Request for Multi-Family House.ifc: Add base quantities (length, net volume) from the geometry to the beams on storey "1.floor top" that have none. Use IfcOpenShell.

First a look at what the model holds.

```python
import ifcopenshell
import ifcopenshell.util.element
import ifcopenshell.util.unit

model = ifcopenshell.open("Multi-Family House.ifc")
print(model.schema)
for unit_type in ("LENGTHUNIT", "AREAUNIT", "VOLUMEUNIT"):
    print(unit_type, ifcopenshell.util.unit.calculate_unit_scale(model, unit_type))
storey = next(s for s in model.by_type("IfcBuildingStorey") if s.Name == "1.floor top")
beams = [e for e in ifcopenshell.util.element.get_decomposition(storey) if e.is_a("IfcBeam")]
for e in sorted(beams, key=lambda e: e.id()):
    print(e.id(), e.is_a(), e.Name, list(ifcopenshell.util.element.get_psets(e, qtos_only=True)), sep=" | ")
```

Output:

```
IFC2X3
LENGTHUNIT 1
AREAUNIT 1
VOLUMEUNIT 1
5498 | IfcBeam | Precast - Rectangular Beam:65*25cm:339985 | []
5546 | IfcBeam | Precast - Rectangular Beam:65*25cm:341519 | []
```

```python
import ifcopenshell
import ifcopenshell.api.pset
import ifcopenshell.geom
import ifcopenshell.util.element
import ifcopenshell.util.shape
import ifcopenshell.util.unit

model = ifcopenshell.open("Multi-Family House.ifc")
unit_scale = ifcopenshell.util.unit.calculate_unit_scale(model)
volume_scale = ifcopenshell.util.unit.calculate_unit_scale(model, "VOLUMEUNIT")
settings = ifcopenshell.geom.settings()

storey = next(s for s in model.by_type("IfcBuildingStorey") if s.Name == "1.floor top")
beams = [e for e in ifcopenshell.util.element.get_decomposition(storey) if e.is_a("IfcBeam")]

for e in sorted(beams, key=lambda e: e.id()):
    if ifcopenshell.util.element.get_psets(e, qtos_only=True, should_inherit=False):
        continue
    # Geometry comes back in metres, in the element's own axes.
    shape = ifcopenshell.geom.create_shape(settings, e)
    values = {
        "Length": ifcopenshell.util.shape.get_max_xyz(shape.geometry) / unit_scale,
        "NetVolume": ifcopenshell.util.shape.get_volume(shape.geometry) / volume_scale,
    }
    qto = ifcopenshell.api.pset.add_qto(model, product=e, name="BaseQuantities")
    ifcopenshell.api.pset.edit_qto(model, qto=qto, properties=values)
    print(e.id(), {k: round(v, 3) for k, v in values.items()})

model.write("Multi-Family House_v2.ifc")
```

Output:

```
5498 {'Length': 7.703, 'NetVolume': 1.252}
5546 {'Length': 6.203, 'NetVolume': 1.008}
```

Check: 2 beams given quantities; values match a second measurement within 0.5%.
